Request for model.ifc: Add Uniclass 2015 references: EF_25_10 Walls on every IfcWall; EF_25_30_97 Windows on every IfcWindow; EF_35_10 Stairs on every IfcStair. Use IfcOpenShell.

First a look at what the model holds.

```python
import ifcopenshell

model = ifcopenshell.open("model.ifc")
print(model.schema)
print("classifications:", [c.Name for c in model.by_type("IfcClassification")])
for ifc_class in ("IfcDoor", "IfcRoof", "IfcStair", "IfcWall", "IfcWindow"):
    print(ifc_class, len(model.by_type(ifc_class)))
```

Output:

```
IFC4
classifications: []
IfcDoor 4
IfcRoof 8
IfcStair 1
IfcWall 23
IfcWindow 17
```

```python
import ifcopenshell
import ifcopenshell.api.classification

model = ifcopenshell.open("model.ifc")

system = ifcopenshell.api.classification.add_classification(model, classification="Uniclass 2015")

codes = {
    "IfcWall": ("EF_25_10", "Walls"),
    "IfcWindow": ("EF_25_30_97", "Windows"),
    "IfcStair": ("EF_35_10", "Stairs"),
}
for ifc_class, (code, name) in codes.items():
    products = model.by_type(ifc_class)
    ifcopenshell.api.classification.add_reference(
        model, products=products, classification=system, identification=code, name=name
    )
    print(code, len(products))

model.write("model-out.ifc")
```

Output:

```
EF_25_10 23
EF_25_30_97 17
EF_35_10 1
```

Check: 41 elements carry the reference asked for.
